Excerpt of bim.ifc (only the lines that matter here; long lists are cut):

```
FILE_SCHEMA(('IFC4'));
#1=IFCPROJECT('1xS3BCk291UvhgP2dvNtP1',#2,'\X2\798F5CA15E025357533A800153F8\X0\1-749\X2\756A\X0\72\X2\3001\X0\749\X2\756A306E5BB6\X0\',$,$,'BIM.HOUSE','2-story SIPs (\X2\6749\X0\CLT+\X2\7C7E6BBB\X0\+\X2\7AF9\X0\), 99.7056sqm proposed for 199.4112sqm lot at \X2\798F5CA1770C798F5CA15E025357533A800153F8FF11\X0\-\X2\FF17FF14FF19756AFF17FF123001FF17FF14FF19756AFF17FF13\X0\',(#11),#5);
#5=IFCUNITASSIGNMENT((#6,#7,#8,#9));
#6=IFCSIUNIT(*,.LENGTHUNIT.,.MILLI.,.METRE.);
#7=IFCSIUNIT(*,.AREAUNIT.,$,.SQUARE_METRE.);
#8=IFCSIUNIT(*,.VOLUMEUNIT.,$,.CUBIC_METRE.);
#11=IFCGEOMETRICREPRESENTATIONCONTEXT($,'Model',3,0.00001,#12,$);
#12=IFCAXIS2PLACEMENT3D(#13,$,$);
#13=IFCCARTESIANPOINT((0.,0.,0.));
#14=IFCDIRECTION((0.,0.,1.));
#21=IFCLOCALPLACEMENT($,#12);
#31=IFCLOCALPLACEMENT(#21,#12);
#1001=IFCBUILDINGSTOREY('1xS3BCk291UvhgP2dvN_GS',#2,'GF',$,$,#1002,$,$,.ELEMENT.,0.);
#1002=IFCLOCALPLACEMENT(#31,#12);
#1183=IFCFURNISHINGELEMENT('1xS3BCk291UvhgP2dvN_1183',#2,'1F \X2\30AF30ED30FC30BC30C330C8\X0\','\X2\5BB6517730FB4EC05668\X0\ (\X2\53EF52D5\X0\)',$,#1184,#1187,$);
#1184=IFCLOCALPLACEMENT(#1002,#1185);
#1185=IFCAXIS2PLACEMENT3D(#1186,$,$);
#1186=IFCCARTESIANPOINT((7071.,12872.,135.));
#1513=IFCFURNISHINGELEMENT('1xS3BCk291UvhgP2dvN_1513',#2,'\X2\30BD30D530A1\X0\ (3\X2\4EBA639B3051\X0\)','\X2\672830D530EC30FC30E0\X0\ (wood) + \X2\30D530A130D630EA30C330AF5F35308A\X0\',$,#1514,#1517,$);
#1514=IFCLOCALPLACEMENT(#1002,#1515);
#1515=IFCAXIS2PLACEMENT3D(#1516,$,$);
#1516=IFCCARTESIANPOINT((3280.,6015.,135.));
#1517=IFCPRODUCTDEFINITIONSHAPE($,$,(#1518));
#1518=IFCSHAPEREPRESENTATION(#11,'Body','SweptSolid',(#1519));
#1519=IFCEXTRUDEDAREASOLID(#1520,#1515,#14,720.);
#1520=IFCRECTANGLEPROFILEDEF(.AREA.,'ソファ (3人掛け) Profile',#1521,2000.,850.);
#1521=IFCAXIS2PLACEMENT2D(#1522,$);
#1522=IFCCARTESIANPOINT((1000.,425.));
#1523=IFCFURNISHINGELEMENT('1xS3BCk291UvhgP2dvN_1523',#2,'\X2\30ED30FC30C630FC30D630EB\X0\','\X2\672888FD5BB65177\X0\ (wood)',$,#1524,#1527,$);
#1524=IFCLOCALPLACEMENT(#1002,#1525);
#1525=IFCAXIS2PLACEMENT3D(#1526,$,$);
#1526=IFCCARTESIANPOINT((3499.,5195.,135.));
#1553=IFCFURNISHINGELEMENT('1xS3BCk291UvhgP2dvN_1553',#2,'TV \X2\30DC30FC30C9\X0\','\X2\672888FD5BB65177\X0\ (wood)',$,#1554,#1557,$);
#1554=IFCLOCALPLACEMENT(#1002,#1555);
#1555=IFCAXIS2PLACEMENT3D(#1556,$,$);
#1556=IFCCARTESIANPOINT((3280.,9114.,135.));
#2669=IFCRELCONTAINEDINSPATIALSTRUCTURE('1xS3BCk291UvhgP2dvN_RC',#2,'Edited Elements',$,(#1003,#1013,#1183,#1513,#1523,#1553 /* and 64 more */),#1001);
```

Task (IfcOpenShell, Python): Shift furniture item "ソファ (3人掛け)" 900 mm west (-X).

```python
import ifcopenshell
import ifcopenshell.api.geometry
import ifcopenshell.util.placement
import ifcopenshell.util.unit

model = ifcopenshell.open("bim.ifc")
unit_scale = ifcopenshell.util.unit.calculate_unit_scale(model)

item = model.by_guid("1xS3BCk291UvhgP2dvN_1513")
matrix = ifcopenshell.util.placement.get_local_placement(item.ObjectPlacement)
matrix[0, 3] -= 0.9 / unit_scale
ifcopenshell.api.geometry.edit_object_placement(model, product=item, matrix=matrix, is_si=False)

print(ifcopenshell.util.placement.get_local_placement(item.ObjectPlacement).round(3) + 0.0)

model.write("bim-out.ifc")
```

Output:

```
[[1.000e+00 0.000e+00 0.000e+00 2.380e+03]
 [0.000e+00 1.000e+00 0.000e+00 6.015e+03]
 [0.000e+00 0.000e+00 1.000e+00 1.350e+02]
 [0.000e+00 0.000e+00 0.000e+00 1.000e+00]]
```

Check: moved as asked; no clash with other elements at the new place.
